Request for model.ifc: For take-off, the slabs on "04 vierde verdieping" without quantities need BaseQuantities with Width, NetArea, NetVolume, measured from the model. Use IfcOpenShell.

First a look at what the model holds.

```python
import ifcopenshell
import ifcopenshell.util.element
import ifcopenshell.util.unit

model = ifcopenshell.open("model.ifc")
print(model.schema)
for unit_type in ("LENGTHUNIT", "AREAUNIT", "VOLUMEUNIT"):
    print(unit_type, ifcopenshell.util.unit.calculate_unit_scale(model, unit_type))
storey = next(s for s in model.by_type("IfcBuildingStorey") if s.Name == "04 vierde verdieping")
slabs = [e for e in ifcopenshell.util.element.get_decomposition(storey) if e.is_a("IfcSlab")]
for e in sorted(slabs, key=lambda e: e.id()):
    print(e.id(), e.is_a(), e.Name, list(ifcopenshell.util.element.get_psets(e, qtos_only=True)), sep=" | ")
```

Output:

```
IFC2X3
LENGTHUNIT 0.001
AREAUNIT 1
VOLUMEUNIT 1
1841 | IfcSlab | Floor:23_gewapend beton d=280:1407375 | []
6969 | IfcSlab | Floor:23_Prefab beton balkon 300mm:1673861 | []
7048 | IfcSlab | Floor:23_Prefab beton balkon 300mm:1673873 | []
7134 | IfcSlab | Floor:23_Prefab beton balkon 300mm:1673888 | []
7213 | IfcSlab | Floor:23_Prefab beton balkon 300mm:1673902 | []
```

```python
import ifcopenshell
import ifcopenshell.api.pset
import ifcopenshell.geom
import ifcopenshell.util.element
import ifcopenshell.util.shape
import ifcopenshell.util.unit

model = ifcopenshell.open("model.ifc")
unit_scale = ifcopenshell.util.unit.calculate_unit_scale(model)
area_scale = ifcopenshell.util.unit.calculate_unit_scale(model, "AREAUNIT")
volume_scale = ifcopenshell.util.unit.calculate_unit_scale(model, "VOLUMEUNIT")
settings = ifcopenshell.geom.settings()

storey = next(s for s in model.by_type("IfcBuildingStorey") if s.Name == "04 vierde verdieping")
slabs = [e for e in ifcopenshell.util.element.get_decomposition(storey) if e.is_a("IfcSlab")]

for e in sorted(slabs, key=lambda e: e.id()):
    if ifcopenshell.util.element.get_psets(e, qtos_only=True, should_inherit=False):
        continue
    # Geometry comes back in metres, in the element's own axes.
    shape = ifcopenshell.geom.create_shape(settings, e)
    values = {
        "Width": ifcopenshell.util.shape.get_z(shape.geometry) / unit_scale,
        "NetArea": ifcopenshell.util.shape.get_footprint_area(shape.geometry) / area_scale,
        "NetVolume": ifcopenshell.util.shape.get_volume(shape.geometry) / volume_scale,
    }
    qto = ifcopenshell.api.pset.add_qto(model, product=e, name="BaseQuantities")
    ifcopenshell.api.pset.edit_qto(model, qto=qto, properties=values)
    print(e.id(), {k: round(v, 3) for k, v in values.items()})

model.write("model-out.ifc")
```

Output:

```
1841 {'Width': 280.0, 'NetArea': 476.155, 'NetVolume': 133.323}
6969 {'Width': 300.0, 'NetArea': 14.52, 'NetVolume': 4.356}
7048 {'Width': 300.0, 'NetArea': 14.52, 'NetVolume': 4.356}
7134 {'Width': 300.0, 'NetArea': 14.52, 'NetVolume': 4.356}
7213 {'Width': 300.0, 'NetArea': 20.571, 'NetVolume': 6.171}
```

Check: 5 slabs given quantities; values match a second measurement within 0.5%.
